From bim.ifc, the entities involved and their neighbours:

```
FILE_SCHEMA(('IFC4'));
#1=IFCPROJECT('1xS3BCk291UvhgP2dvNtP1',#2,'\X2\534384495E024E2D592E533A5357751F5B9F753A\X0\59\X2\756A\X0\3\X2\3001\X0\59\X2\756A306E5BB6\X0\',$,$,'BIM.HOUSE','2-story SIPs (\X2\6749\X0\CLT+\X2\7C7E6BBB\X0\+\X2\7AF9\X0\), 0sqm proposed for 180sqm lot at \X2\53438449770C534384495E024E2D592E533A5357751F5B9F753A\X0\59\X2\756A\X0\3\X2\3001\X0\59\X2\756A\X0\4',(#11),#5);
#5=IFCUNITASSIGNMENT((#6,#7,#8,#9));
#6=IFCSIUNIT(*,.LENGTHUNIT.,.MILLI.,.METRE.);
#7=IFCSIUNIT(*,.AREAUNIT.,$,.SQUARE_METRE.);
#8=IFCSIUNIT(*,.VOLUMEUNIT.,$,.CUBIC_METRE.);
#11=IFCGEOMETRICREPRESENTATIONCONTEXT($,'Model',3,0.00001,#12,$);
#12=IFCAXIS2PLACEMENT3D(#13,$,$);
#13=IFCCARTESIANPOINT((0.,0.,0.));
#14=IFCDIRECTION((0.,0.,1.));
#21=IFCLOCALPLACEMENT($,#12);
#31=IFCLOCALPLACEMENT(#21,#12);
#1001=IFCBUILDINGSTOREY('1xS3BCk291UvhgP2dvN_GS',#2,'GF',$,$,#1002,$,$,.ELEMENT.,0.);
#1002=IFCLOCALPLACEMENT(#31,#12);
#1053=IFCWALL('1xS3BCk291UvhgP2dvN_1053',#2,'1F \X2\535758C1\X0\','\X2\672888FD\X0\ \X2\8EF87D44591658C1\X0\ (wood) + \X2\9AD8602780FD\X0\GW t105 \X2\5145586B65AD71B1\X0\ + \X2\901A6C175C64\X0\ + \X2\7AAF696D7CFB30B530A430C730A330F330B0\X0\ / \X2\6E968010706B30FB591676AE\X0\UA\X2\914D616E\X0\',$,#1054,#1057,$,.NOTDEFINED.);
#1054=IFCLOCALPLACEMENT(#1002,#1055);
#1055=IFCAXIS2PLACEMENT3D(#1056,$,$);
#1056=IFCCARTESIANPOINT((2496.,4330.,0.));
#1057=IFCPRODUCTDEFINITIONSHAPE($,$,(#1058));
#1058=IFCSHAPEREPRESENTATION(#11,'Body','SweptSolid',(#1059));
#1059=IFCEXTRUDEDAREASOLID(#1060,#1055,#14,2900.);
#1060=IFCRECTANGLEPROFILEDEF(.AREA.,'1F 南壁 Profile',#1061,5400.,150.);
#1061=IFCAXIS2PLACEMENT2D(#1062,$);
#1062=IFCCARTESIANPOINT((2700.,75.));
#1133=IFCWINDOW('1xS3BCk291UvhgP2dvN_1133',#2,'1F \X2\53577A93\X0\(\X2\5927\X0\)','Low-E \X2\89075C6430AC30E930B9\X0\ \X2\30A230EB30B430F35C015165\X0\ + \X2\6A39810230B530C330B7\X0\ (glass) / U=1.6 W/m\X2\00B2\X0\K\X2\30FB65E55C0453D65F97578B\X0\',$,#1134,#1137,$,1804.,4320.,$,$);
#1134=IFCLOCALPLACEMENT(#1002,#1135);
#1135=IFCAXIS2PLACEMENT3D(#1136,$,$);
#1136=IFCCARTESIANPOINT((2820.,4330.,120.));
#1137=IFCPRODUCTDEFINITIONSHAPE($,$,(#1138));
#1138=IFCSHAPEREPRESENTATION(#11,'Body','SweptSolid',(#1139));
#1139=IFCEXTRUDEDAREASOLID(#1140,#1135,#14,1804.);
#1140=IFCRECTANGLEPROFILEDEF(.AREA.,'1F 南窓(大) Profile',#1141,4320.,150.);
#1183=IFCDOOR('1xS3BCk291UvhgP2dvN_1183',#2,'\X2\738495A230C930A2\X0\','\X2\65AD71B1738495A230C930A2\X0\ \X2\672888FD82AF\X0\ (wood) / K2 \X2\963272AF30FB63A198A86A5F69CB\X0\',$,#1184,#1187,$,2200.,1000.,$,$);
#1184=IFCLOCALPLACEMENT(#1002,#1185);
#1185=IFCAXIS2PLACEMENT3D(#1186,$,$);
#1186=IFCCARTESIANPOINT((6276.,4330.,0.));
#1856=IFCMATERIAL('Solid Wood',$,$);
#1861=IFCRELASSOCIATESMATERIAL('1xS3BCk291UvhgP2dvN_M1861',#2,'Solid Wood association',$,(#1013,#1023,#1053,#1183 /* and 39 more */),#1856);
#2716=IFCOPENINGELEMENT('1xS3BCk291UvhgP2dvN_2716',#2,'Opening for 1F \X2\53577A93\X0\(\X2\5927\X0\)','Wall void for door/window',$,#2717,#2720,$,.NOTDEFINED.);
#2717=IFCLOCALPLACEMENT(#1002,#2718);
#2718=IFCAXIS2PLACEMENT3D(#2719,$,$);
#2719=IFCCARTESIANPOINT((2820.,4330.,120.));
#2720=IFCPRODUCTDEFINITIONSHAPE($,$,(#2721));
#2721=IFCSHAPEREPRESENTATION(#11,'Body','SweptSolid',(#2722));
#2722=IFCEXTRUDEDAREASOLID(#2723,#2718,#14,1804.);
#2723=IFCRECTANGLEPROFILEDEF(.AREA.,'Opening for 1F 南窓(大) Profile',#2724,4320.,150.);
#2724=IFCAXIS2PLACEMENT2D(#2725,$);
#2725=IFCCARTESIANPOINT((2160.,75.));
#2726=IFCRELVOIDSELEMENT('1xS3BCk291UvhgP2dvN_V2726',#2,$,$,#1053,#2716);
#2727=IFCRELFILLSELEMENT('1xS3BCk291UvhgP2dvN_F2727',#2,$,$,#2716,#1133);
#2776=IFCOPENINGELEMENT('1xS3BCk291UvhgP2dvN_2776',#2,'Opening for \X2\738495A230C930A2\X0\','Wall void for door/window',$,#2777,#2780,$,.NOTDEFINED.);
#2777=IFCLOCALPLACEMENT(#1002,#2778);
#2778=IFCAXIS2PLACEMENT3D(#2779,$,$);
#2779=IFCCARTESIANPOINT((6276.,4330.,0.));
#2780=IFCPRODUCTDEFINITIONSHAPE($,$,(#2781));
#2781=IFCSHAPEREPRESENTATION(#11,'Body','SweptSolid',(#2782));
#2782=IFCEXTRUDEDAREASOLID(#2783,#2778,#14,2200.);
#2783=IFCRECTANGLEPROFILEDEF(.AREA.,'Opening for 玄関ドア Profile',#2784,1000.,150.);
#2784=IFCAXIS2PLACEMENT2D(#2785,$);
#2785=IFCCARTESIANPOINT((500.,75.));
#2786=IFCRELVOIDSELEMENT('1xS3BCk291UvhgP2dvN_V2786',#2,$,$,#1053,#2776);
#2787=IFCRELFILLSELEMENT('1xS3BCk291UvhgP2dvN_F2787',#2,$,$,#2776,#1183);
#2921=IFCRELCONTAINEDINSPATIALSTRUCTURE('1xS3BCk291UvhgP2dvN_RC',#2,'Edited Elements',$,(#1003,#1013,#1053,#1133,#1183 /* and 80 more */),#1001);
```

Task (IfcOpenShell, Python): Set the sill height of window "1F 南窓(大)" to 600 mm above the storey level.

```python
import numpy as np
import ifcopenshell
import ifcopenshell.api.geometry
import ifcopenshell.geom
import ifcopenshell.util.element
import ifcopenshell.util.placement
import ifcopenshell.util.shape
import ifcopenshell.util.unit

model = ifcopenshell.open("bim.ifc")
unit_scale = ifcopenshell.util.unit.calculate_unit_scale(model)

window = model.by_guid("1xS3BCk291UvhgP2dvN_1133")
opening = window.FillsVoids[0].RelatingOpeningElement
storey = ifcopenshell.util.element.get_container(window, ifc_class="IfcBuildingStorey")
level = ifcopenshell.util.placement.get_local_placement(storey.ObjectPlacement)[2, 3]

# The opening's origin need not be at the sill, so measure its lowest point.
shape = ifcopenshell.geom.create_shape(ifcopenshell.geom.settings(), opening)
bottom = ifcopenshell.util.shape.get_shape_bottom_elevation(shape, shape.geometry) / unit_scale
dz = level + 600.0 - bottom

shift = np.array([0.0, 0.0, dz])
# The window is not placed relative to its opening, so move both.
for product in (opening, window):
    matrix = ifcopenshell.util.placement.get_local_placement(product.ObjectPlacement)
    matrix[:3, 3] += shift
    ifcopenshell.api.geometry.edit_object_placement(model, product=product, matrix=matrix, is_si=False)

print(f"moved by {dz * unit_scale:+.3f} m")

model.write("bim_rev.ifc")
```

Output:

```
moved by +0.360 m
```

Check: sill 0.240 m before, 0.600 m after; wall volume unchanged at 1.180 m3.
